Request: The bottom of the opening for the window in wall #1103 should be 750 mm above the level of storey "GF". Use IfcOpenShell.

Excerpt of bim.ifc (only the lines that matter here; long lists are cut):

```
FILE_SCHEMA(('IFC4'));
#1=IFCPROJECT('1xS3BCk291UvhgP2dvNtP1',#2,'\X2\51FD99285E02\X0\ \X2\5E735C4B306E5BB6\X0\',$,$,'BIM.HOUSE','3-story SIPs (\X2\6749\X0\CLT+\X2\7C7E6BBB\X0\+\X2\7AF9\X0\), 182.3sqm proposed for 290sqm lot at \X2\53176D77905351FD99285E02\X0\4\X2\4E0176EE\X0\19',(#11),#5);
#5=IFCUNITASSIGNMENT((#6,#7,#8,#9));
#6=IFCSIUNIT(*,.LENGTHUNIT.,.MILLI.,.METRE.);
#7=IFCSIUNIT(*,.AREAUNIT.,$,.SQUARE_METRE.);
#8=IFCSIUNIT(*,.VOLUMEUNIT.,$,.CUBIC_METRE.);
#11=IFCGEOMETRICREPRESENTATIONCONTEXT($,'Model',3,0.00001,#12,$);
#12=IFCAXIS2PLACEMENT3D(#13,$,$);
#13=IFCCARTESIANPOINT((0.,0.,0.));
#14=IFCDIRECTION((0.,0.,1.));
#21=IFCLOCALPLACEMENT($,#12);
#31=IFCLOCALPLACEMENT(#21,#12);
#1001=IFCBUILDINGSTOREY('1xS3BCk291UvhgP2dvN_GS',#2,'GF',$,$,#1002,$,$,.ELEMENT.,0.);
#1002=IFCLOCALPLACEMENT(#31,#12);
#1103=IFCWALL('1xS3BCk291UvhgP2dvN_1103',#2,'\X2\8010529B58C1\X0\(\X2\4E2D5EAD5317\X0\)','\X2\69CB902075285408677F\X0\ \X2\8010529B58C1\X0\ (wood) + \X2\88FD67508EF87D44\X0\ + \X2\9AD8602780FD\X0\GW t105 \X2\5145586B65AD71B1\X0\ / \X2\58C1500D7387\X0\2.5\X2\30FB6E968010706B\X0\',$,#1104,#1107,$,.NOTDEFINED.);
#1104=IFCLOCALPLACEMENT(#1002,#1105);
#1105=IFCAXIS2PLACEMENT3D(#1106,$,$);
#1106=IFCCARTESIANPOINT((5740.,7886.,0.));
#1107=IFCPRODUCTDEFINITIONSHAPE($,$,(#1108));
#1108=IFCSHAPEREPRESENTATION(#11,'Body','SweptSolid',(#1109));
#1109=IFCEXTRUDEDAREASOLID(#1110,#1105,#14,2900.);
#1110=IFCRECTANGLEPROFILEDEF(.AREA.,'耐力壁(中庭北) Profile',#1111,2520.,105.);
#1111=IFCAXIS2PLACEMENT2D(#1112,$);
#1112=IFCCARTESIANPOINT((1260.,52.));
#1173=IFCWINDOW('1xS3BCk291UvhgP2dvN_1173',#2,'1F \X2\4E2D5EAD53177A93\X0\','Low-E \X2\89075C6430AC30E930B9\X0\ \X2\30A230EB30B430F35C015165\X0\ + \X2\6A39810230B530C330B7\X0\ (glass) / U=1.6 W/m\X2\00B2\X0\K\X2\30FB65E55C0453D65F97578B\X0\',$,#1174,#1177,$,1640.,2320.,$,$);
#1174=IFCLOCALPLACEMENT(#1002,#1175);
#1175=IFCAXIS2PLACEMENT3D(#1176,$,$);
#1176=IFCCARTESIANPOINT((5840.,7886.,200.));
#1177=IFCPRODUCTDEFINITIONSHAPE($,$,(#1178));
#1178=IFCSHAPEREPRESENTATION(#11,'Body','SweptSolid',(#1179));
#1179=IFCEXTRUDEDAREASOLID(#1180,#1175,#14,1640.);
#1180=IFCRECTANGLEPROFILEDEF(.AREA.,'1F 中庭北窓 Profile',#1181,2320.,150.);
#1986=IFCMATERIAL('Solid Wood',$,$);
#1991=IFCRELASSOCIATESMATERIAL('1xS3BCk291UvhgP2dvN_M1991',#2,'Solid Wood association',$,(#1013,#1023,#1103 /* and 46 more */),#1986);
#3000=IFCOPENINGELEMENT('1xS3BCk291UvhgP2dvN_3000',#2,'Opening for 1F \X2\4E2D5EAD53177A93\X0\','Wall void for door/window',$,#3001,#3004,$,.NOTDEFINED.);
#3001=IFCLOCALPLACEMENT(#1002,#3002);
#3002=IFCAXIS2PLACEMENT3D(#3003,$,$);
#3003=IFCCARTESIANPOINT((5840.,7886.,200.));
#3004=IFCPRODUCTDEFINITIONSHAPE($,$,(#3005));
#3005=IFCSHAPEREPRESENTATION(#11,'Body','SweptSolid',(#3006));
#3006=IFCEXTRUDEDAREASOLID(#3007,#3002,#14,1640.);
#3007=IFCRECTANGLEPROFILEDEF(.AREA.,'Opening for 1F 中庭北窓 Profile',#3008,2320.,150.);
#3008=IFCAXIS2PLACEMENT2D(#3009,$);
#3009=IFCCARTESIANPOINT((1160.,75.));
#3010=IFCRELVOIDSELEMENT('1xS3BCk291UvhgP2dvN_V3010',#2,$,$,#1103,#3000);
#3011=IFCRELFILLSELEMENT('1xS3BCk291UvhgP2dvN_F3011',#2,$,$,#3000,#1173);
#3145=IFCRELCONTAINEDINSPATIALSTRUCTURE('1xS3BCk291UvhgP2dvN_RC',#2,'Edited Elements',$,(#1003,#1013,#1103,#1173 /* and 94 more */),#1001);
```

```python
import numpy as np
import ifcopenshell
import ifcopenshell.api.geometry
import ifcopenshell.geom
import ifcopenshell.util.element
import ifcopenshell.util.placement
import ifcopenshell.util.shape
import ifcopenshell.util.unit

model = ifcopenshell.open("bim.ifc")
unit_scale = ifcopenshell.util.unit.calculate_unit_scale(model)

window = model.by_guid("1xS3BCk291UvhgP2dvN_1173")
opening = window.FillsVoids[0].RelatingOpeningElement
storey = ifcopenshell.util.element.get_container(window, ifc_class="IfcBuildingStorey")
level = ifcopenshell.util.placement.get_local_placement(storey.ObjectPlacement)[2, 3]

# The opening's origin need not be at the sill, so measure its lowest point.
shape = ifcopenshell.geom.create_shape(ifcopenshell.geom.settings(), opening)
bottom = ifcopenshell.util.shape.get_shape_bottom_elevation(shape, shape.geometry) / unit_scale
dz = level + 0.75 / unit_scale - bottom

shift = np.array([0.0, 0.0, dz])
# The window is not placed relative to its opening, so move both.
for product in (opening, window):
    matrix = ifcopenshell.util.placement.get_local_placement(product.ObjectPlacement)
    matrix[:3, 3] += shift
    ifcopenshell.api.geometry.edit_object_placement(model, product=product, matrix=matrix, is_si=False)

print(f"moved by {dz * unit_scale:+.3f} m")

model.write("bim-out.ifc")
```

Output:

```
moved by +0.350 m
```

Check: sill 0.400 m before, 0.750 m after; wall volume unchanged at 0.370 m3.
